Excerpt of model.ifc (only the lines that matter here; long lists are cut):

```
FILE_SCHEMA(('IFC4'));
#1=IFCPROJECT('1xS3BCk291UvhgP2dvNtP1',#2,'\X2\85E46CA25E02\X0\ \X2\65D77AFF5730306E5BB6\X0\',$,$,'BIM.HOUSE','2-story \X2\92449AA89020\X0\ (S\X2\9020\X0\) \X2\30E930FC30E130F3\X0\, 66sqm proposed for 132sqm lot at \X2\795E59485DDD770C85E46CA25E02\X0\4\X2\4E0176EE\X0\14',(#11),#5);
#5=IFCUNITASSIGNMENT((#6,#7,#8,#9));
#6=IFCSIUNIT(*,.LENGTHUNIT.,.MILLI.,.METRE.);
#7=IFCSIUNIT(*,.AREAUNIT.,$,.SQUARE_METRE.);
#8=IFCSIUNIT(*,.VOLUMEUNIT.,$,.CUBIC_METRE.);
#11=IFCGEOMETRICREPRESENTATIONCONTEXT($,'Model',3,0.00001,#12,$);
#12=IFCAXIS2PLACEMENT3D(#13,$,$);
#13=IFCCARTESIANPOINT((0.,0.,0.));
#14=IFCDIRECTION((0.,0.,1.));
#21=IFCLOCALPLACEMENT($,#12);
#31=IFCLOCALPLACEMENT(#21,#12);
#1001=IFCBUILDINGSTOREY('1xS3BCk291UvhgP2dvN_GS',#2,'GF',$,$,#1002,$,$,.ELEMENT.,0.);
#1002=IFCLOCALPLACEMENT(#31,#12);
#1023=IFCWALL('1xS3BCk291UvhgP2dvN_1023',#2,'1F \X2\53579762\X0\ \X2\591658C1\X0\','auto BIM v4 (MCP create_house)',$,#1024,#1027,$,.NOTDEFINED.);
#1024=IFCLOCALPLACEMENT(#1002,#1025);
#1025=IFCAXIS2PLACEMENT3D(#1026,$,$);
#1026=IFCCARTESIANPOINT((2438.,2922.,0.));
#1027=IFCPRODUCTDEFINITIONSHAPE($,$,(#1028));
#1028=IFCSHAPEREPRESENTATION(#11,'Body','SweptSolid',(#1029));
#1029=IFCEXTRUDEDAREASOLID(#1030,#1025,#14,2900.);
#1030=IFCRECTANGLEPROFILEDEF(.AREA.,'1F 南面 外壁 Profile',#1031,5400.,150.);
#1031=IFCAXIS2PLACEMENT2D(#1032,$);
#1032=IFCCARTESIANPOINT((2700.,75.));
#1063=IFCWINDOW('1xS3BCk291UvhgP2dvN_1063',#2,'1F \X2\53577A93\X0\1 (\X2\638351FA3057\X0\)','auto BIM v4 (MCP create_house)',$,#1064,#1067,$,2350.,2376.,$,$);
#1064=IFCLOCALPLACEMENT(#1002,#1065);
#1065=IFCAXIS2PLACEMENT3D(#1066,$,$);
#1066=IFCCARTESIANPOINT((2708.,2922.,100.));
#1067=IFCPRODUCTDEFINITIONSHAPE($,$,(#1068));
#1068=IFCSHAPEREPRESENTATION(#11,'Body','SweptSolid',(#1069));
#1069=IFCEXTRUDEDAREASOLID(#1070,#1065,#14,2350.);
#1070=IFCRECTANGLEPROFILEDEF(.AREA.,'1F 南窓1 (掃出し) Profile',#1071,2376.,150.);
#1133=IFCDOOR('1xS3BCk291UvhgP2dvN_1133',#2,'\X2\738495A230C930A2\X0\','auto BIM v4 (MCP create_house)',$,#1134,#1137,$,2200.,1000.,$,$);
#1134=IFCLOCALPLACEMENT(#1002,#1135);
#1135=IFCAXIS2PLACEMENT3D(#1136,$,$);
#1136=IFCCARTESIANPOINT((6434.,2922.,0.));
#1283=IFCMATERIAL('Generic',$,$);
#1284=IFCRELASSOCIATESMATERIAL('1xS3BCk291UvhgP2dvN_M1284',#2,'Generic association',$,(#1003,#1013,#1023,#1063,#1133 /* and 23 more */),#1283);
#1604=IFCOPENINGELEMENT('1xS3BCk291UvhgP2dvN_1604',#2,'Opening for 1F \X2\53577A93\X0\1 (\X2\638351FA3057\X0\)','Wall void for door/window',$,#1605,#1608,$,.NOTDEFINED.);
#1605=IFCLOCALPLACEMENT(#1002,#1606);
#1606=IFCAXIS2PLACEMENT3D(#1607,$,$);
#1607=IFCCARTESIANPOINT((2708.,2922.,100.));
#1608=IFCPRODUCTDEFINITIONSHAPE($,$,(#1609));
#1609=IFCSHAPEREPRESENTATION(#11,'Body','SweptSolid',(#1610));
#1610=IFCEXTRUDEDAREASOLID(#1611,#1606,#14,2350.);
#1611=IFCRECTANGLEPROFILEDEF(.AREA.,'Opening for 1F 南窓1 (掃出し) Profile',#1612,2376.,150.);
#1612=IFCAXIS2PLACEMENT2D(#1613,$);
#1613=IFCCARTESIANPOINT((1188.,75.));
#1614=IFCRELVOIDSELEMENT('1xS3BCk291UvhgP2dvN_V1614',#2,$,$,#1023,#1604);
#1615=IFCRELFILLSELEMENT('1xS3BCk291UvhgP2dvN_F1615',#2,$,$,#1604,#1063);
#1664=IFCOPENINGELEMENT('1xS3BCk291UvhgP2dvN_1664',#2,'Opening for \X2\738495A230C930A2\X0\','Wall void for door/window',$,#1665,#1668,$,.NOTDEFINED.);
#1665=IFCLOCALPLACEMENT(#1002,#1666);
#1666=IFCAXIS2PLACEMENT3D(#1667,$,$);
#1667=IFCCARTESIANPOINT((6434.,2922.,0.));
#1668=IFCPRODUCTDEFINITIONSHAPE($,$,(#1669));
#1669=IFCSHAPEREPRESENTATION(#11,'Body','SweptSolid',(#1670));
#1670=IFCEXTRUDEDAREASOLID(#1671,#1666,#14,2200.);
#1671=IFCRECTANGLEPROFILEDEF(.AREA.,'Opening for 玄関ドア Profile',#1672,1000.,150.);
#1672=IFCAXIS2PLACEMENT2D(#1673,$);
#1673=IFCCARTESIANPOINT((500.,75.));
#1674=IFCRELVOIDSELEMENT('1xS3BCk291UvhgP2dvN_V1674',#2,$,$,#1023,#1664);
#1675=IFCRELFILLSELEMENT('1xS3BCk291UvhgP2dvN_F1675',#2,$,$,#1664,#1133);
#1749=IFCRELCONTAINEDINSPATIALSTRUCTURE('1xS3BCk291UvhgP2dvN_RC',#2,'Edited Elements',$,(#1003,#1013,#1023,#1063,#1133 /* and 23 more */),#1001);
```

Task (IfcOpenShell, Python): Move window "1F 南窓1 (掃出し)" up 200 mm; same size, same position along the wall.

```python
import numpy as np
import ifcopenshell
import ifcopenshell.api.geometry
import ifcopenshell.util.placement
import ifcopenshell.util.unit

model = ifcopenshell.open("model.ifc")
unit_scale = ifcopenshell.util.unit.calculate_unit_scale(model)

window = model.by_guid("1xS3BCk291UvhgP2dvN_1063")
opening = window.FillsVoids[0].RelatingOpeningElement
dz = 0.2 / unit_scale

shift = np.array([0.0, 0.0, dz])
# The window is not placed relative to its opening, so move both.
for product in (opening, window):
    matrix = ifcopenshell.util.placement.get_local_placement(product.ObjectPlacement)
    matrix[:3, 3] += shift
    ifcopenshell.api.geometry.edit_object_placement(model, product=product, matrix=matrix, is_si=False)

print(f"moved by {dz * unit_scale:+.3f} m")

model.write("model_v2.ifc")
```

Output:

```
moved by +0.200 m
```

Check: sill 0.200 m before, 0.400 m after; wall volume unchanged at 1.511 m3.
